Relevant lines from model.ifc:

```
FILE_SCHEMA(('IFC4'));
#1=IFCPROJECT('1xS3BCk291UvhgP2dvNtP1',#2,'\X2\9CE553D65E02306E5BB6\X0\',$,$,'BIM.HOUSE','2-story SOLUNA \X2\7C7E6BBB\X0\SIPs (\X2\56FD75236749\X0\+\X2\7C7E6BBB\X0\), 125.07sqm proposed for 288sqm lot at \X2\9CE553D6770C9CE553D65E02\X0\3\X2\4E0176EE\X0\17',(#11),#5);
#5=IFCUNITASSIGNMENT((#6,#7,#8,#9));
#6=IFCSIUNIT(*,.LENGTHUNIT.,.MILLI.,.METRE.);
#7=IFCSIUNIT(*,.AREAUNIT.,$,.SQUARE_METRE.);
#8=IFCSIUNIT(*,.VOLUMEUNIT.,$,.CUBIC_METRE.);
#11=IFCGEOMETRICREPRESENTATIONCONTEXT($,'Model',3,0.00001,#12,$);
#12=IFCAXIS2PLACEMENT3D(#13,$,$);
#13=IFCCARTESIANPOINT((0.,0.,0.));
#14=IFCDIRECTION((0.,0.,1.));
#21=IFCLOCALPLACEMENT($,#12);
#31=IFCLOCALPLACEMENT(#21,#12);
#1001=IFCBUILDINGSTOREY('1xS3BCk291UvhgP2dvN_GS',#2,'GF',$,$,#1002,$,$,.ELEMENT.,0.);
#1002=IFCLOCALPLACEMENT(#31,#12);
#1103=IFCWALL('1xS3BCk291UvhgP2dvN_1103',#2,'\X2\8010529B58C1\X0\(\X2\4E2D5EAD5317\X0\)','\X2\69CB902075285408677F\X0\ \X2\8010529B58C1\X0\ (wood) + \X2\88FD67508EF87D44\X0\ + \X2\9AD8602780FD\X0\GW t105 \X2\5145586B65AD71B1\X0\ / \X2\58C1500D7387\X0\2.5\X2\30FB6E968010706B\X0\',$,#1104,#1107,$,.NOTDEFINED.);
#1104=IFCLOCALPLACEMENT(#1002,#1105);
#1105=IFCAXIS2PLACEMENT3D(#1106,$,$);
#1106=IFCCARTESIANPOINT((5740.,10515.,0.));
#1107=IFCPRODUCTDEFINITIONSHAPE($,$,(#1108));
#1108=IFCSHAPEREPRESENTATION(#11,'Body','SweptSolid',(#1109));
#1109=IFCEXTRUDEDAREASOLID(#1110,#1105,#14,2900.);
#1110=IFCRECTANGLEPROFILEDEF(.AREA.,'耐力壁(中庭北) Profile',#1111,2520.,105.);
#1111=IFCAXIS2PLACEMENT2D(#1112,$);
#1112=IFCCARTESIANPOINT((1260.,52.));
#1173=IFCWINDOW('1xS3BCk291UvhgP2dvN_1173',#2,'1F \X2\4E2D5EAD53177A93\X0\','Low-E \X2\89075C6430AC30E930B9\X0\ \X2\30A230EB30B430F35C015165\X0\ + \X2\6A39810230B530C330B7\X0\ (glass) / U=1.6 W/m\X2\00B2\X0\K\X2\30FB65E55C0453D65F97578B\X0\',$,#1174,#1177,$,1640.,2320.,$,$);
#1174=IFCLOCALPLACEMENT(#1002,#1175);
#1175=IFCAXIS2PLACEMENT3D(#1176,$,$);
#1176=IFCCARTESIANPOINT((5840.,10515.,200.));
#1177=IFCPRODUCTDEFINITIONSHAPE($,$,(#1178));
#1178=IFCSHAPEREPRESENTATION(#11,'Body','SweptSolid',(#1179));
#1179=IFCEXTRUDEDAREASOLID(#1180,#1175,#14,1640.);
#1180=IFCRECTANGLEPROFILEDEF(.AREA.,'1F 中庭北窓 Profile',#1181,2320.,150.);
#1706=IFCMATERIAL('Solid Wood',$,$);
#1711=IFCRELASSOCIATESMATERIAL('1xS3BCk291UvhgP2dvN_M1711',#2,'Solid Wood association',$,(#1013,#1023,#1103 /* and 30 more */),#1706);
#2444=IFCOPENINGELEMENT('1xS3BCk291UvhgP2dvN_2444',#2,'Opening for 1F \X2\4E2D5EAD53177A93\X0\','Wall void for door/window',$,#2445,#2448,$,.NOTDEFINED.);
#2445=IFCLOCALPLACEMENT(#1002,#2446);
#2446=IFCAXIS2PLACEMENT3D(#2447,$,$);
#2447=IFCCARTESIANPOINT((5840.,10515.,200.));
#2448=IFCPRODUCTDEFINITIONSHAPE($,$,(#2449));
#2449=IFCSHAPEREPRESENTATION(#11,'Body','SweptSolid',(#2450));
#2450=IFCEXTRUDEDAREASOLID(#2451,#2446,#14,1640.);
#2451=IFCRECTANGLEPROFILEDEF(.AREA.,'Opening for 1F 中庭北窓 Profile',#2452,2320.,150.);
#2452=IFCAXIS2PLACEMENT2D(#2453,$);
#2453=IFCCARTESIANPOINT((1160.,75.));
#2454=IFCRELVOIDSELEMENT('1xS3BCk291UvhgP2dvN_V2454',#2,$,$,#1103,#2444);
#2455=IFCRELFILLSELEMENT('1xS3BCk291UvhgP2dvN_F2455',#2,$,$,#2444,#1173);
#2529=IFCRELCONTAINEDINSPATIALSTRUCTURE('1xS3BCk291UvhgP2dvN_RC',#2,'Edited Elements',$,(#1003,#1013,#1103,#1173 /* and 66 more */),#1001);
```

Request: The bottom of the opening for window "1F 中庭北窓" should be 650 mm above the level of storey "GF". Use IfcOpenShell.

```python
import numpy as np
import ifcopenshell
import ifcopenshell.api.geometry
import ifcopenshell.geom
import ifcopenshell.util.element
import ifcopenshell.util.placement
import ifcopenshell.util.shape
import ifcopenshell.util.unit

model = ifcopenshell.open("model.ifc")
unit_scale = ifcopenshell.util.unit.calculate_unit_scale(model)

window = model.by_guid("1xS3BCk291UvhgP2dvN_1173")
opening = window.FillsVoids[0].RelatingOpeningElement
storey = ifcopenshell.util.element.get_container(window, ifc_class="IfcBuildingStorey")
level = ifcopenshell.util.placement.get_local_placement(storey.ObjectPlacement)[2, 3]

# The opening's origin need not be at the sill, so measure its lowest point.
shape = ifcopenshell.geom.create_shape(ifcopenshell.geom.settings(), opening)
bottom = ifcopenshell.util.shape.get_shape_bottom_elevation(shape, shape.geometry) / unit_scale
dz = level + 0.65 / unit_scale - bottom

shift = np.array([0.0, 0.0, dz])
# The window is not placed relative to its opening, so move both.
for product in (opening, window):
    matrix = ifcopenshell.util.placement.get_local_placement(product.ObjectPlacement)
    matrix[:3, 3] += shift
    ifcopenshell.api.geometry.edit_object_placement(model, product=product, matrix=matrix, is_si=False)

print(f"moved by {dz * unit_scale:+.3f} m")

model.write("model_edited.ifc")
```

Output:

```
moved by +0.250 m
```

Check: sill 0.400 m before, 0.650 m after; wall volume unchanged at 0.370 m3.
